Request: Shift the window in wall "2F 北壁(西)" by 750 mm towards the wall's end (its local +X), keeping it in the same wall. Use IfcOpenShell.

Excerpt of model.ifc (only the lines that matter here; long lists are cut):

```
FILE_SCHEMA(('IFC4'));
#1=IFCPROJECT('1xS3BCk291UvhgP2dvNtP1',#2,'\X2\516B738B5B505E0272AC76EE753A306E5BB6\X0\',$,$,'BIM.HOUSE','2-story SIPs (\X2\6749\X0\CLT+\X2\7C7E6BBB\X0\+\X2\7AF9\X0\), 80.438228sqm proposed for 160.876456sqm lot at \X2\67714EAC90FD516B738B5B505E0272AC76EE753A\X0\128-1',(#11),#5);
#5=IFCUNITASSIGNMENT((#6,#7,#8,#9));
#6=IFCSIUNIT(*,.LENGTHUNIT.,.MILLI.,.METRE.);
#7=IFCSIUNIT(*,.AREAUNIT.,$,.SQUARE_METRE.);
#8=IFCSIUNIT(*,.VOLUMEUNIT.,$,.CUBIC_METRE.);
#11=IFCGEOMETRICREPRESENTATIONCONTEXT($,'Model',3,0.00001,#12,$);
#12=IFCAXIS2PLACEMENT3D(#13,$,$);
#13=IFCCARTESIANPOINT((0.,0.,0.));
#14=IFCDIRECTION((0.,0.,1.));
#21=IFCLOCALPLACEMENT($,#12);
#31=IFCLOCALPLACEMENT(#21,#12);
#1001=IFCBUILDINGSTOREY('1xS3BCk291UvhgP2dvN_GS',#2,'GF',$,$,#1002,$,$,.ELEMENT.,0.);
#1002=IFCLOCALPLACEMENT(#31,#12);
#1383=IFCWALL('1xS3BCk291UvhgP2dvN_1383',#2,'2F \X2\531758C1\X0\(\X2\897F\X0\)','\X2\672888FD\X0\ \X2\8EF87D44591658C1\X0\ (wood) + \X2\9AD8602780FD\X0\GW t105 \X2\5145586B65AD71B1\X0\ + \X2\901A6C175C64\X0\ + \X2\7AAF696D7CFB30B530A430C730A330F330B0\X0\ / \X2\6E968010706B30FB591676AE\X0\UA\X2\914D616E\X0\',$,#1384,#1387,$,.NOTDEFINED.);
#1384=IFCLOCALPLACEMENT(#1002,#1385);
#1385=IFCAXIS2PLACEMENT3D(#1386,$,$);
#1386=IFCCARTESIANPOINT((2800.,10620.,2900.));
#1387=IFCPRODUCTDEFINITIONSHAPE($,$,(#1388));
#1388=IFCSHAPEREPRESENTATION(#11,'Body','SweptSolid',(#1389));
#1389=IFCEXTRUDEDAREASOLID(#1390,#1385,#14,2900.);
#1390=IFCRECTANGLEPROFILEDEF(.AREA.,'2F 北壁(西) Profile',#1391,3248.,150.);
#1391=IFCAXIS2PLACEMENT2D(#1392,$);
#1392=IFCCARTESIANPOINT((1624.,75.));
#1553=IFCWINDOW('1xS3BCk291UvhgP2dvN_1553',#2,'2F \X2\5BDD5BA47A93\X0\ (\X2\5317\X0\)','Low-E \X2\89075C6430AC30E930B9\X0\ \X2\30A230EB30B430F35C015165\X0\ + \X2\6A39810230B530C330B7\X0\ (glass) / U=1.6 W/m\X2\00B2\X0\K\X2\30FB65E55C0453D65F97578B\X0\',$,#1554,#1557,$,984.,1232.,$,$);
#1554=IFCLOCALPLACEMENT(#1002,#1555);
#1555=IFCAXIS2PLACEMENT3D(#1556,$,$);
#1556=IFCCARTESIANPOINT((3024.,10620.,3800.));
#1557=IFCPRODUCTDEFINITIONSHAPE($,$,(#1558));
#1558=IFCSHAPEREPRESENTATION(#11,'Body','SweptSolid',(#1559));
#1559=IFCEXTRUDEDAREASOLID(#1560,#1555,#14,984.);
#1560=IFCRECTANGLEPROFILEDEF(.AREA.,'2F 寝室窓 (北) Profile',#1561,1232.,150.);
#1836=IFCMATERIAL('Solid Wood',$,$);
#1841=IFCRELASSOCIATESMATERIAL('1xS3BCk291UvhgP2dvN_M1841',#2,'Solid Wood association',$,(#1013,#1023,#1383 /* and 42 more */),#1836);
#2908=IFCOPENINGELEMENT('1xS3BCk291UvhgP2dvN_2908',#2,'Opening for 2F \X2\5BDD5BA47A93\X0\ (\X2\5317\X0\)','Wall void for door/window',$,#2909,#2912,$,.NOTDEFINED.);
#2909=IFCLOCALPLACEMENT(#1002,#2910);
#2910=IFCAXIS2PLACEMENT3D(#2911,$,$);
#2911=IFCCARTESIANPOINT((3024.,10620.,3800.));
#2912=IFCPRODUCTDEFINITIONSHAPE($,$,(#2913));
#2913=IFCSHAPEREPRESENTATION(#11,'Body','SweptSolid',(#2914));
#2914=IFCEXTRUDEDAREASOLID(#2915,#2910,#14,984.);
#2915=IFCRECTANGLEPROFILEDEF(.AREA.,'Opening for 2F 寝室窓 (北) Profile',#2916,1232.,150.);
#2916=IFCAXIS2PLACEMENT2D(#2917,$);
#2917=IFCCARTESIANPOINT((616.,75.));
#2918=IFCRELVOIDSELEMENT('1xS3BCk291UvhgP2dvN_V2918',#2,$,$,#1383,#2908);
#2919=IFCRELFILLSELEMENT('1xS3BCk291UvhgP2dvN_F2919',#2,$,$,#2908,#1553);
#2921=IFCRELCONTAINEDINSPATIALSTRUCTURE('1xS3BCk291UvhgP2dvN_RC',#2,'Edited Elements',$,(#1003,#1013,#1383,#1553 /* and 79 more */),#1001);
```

```python
import ifcopenshell
import ifcopenshell.api.geometry
import ifcopenshell.util.placement

model = ifcopenshell.open("model.ifc")

window = model.by_guid("1xS3BCk291UvhgP2dvN_1553")
opening = window.FillsVoids[0].RelatingOpeningElement
wall = opening.VoidsElements[0].RelatingBuildingElement

wall_matrix = ifcopenshell.util.placement.get_local_placement(wall.ObjectPlacement)
shift = wall_matrix[:3, 0] * 750.0
before = ifcopenshell.util.placement.get_local_placement(window.ObjectPlacement)[:3, 3].copy()

# The window is not placed relative to its opening, so move both.
for product in (opening, window):
    matrix = ifcopenshell.util.placement.get_local_placement(product.ObjectPlacement)
    matrix[:3, 3] += shift
    ifcopenshell.api.geometry.edit_object_placement(model, product=product, matrix=matrix, is_si=False)

after = ifcopenshell.util.placement.get_local_placement(window.ObjectPlacement)[:3, 3]
print("window moved by", (after - before).round(3) + 0.0)

model.write("model-out.ifc")
```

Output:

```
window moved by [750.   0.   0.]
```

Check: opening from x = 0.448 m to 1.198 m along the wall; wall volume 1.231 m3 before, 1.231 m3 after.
